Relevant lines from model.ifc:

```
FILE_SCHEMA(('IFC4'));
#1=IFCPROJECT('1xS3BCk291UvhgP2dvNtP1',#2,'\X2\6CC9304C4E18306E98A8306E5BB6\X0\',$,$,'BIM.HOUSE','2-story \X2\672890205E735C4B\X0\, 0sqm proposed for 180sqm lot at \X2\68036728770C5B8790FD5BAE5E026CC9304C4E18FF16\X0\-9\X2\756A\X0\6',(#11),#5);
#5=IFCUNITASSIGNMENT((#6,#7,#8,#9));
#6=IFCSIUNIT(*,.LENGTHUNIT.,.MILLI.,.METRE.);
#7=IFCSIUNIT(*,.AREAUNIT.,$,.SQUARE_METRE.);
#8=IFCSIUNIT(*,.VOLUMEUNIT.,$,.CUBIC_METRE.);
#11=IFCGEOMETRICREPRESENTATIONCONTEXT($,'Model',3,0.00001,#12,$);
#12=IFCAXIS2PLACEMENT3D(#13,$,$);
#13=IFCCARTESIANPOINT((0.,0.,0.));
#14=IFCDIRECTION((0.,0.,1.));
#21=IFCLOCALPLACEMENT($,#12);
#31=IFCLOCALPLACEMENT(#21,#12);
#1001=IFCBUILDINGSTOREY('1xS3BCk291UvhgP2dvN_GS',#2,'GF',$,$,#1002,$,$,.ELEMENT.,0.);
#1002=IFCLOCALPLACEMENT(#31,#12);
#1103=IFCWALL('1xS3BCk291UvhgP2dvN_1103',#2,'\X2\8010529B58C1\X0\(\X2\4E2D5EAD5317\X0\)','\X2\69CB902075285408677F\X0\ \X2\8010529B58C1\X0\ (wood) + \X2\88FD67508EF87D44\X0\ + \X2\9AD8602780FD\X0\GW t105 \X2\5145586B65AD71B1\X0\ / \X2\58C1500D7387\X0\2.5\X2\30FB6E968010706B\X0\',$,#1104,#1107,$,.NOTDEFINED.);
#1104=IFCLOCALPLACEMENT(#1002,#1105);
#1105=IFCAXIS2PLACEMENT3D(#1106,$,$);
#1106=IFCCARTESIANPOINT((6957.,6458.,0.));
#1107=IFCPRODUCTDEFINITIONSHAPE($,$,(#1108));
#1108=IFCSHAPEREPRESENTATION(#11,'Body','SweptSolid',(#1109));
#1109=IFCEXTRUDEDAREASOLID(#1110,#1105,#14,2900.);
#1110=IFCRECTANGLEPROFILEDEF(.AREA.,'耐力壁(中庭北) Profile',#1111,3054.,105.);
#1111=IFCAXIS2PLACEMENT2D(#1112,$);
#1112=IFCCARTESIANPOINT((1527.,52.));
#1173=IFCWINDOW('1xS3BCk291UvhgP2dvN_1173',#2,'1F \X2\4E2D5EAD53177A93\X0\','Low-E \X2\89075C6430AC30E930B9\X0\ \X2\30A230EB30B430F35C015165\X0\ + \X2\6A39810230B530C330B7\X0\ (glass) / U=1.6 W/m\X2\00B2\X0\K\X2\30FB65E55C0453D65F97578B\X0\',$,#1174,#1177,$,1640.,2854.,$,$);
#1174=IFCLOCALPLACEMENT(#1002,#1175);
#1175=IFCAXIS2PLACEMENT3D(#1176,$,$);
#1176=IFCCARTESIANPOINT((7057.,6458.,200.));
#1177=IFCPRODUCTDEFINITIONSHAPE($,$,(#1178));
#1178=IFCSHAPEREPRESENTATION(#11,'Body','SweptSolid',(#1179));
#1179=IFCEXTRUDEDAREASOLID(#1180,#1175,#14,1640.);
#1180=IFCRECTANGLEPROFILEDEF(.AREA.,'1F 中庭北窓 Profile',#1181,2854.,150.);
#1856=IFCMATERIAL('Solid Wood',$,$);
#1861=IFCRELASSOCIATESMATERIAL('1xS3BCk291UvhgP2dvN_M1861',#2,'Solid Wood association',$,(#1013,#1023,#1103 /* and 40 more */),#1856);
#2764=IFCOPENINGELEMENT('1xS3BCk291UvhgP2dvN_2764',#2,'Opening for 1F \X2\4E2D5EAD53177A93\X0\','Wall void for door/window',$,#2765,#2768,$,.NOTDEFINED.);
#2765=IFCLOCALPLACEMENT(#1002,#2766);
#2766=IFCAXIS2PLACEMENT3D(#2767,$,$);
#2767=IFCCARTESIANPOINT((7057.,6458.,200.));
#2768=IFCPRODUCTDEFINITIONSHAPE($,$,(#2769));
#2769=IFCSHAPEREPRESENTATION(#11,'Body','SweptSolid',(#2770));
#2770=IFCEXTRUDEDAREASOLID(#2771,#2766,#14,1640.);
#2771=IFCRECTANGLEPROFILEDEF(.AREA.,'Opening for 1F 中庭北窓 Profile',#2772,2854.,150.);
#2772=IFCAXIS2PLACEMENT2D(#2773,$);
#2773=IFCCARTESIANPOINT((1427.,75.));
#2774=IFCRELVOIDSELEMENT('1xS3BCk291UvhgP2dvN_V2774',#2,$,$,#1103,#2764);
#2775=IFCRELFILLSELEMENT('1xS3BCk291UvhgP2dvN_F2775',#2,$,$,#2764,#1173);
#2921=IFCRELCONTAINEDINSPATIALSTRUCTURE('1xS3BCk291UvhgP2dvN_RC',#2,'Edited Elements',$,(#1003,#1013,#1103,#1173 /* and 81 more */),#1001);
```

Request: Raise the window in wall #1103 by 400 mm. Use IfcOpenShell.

```python
import numpy as np
import ifcopenshell
import ifcopenshell.api.geometry
import ifcopenshell.util.placement
import ifcopenshell.util.unit

model = ifcopenshell.open("model.ifc")
unit_scale = ifcopenshell.util.unit.calculate_unit_scale(model)

window = model.by_id(1173)
opening = window.FillsVoids[0].RelatingOpeningElement
dz = 0.4 / unit_scale

shift = np.array([0.0, 0.0, dz])
# The window is not placed relative to its opening, so move both.
for product in (opening, window):
    matrix = ifcopenshell.util.placement.get_local_placement(product.ObjectPlacement)
    matrix[:3, 3] += shift
    ifcopenshell.api.geometry.edit_object_placement(model, product=product, matrix=matrix, is_si=False)

print(f"moved by {dz * unit_scale:+.3f} m")

model.write("model_v2.ifc")
```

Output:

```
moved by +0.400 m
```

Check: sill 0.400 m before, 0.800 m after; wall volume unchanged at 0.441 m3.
